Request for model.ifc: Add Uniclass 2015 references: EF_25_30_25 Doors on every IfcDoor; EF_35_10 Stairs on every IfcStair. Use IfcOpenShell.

First a look at what the model holds.

```python
import ifcopenshell

model = ifcopenshell.open("model.ifc")
print(model.schema)
print("classifications:", [c.Name for c in model.by_type("IfcClassification")])
for ifc_class in ("IfcDoor", "IfcRoof", "IfcStair", "IfcWall", "IfcWindow"):
    print(ifc_class, len(model.by_type(ifc_class)))
```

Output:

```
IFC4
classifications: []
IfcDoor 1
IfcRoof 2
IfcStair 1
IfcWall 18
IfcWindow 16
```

```python
import ifcopenshell
import ifcopenshell.api.classification

model = ifcopenshell.open("model.ifc")

system = ifcopenshell.api.classification.add_classification(model, classification="Uniclass 2015")

codes = {
    "IfcDoor": ("EF_25_30_25", "Doors"),
    "IfcStair": ("EF_35_10", "Stairs"),
}
for ifc_class, (code, name) in codes.items():
    products = model.by_type(ifc_class)
    ifcopenshell.api.classification.add_reference(
        model, products=products, classification=system, identification=code, name=name
    )
    print(code, len(products))

model.write("model_updated.ifc")
```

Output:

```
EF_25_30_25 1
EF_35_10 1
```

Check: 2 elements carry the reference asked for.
